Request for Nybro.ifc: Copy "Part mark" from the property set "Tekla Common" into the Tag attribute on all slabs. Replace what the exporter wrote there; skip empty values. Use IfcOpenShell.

First a look at what the model holds.

```python
import ifcopenshell
import ifcopenshell.util.element

model = ifcopenshell.open("Nybro.ifc")
print(model.schema)
slabs = model.by_type("IfcSlab")
print(len(slabs), "slabs")
for e in slabs[:8]:
    source = ifcopenshell.util.element.get_pset(e, "Tekla Common", "Part mark")
    target = e.Tag
    print(e.id(), repr(source), repr(target), sep=" | ")
```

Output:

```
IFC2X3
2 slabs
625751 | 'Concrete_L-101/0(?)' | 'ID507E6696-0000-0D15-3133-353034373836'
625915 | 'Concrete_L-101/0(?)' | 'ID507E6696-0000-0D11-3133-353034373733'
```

```python
import ifcopenshell
import ifcopenshell.util.element

model = ifcopenshell.open("Nybro.ifc")

count = 0
for e in model.by_type("IfcSlab"):
    value = ifcopenshell.util.element.get_pset(e, "Tekla Common", "Part mark")
    current = e.Tag
    if not value or not value.strip() or current == value:
        continue
    e.Tag = value
    count += 1

print(count, "slabs updated")

model.write("Nybro_rev.ifc")
```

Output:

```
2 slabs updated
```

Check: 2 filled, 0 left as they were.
